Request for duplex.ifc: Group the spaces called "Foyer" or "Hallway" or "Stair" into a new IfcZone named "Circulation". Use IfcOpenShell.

First a look at what the model holds.

```python
import ifcopenshell

model = ifcopenshell.open("duplex.ifc")
print(model.schema)
seen = {}
for space in model.by_type("IfcSpace"):
    seen[space.LongName] = seen.get(space.LongName, 0) + 1
for name, count in sorted(seen.items(), key=str):
    print(count, "x", name)
print("zones:", [z.Name for z in model.by_type("IfcZone")][:20])
```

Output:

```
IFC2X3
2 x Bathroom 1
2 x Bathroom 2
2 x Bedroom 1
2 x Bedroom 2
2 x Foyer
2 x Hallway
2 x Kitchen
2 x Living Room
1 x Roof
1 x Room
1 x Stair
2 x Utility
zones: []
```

```python
import ifcopenshell
import ifcopenshell.api.group
import ifcopenshell.api.root

model = ifcopenshell.open("duplex.ifc")

names = {"Foyer", "Hallway", "Stair"}
spaces = [s for s in model.by_type("IfcSpace") if s.LongName in names]

zone = ifcopenshell.api.root.create_entity(model, ifc_class="IfcZone", name="Circulation")
ifcopenshell.api.group.assign_group(model, products=spaces, group=zone)
print(len(spaces), "spaces in", zone.Name)

model.write("duplex-out.ifc")
```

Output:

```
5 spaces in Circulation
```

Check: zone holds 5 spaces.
